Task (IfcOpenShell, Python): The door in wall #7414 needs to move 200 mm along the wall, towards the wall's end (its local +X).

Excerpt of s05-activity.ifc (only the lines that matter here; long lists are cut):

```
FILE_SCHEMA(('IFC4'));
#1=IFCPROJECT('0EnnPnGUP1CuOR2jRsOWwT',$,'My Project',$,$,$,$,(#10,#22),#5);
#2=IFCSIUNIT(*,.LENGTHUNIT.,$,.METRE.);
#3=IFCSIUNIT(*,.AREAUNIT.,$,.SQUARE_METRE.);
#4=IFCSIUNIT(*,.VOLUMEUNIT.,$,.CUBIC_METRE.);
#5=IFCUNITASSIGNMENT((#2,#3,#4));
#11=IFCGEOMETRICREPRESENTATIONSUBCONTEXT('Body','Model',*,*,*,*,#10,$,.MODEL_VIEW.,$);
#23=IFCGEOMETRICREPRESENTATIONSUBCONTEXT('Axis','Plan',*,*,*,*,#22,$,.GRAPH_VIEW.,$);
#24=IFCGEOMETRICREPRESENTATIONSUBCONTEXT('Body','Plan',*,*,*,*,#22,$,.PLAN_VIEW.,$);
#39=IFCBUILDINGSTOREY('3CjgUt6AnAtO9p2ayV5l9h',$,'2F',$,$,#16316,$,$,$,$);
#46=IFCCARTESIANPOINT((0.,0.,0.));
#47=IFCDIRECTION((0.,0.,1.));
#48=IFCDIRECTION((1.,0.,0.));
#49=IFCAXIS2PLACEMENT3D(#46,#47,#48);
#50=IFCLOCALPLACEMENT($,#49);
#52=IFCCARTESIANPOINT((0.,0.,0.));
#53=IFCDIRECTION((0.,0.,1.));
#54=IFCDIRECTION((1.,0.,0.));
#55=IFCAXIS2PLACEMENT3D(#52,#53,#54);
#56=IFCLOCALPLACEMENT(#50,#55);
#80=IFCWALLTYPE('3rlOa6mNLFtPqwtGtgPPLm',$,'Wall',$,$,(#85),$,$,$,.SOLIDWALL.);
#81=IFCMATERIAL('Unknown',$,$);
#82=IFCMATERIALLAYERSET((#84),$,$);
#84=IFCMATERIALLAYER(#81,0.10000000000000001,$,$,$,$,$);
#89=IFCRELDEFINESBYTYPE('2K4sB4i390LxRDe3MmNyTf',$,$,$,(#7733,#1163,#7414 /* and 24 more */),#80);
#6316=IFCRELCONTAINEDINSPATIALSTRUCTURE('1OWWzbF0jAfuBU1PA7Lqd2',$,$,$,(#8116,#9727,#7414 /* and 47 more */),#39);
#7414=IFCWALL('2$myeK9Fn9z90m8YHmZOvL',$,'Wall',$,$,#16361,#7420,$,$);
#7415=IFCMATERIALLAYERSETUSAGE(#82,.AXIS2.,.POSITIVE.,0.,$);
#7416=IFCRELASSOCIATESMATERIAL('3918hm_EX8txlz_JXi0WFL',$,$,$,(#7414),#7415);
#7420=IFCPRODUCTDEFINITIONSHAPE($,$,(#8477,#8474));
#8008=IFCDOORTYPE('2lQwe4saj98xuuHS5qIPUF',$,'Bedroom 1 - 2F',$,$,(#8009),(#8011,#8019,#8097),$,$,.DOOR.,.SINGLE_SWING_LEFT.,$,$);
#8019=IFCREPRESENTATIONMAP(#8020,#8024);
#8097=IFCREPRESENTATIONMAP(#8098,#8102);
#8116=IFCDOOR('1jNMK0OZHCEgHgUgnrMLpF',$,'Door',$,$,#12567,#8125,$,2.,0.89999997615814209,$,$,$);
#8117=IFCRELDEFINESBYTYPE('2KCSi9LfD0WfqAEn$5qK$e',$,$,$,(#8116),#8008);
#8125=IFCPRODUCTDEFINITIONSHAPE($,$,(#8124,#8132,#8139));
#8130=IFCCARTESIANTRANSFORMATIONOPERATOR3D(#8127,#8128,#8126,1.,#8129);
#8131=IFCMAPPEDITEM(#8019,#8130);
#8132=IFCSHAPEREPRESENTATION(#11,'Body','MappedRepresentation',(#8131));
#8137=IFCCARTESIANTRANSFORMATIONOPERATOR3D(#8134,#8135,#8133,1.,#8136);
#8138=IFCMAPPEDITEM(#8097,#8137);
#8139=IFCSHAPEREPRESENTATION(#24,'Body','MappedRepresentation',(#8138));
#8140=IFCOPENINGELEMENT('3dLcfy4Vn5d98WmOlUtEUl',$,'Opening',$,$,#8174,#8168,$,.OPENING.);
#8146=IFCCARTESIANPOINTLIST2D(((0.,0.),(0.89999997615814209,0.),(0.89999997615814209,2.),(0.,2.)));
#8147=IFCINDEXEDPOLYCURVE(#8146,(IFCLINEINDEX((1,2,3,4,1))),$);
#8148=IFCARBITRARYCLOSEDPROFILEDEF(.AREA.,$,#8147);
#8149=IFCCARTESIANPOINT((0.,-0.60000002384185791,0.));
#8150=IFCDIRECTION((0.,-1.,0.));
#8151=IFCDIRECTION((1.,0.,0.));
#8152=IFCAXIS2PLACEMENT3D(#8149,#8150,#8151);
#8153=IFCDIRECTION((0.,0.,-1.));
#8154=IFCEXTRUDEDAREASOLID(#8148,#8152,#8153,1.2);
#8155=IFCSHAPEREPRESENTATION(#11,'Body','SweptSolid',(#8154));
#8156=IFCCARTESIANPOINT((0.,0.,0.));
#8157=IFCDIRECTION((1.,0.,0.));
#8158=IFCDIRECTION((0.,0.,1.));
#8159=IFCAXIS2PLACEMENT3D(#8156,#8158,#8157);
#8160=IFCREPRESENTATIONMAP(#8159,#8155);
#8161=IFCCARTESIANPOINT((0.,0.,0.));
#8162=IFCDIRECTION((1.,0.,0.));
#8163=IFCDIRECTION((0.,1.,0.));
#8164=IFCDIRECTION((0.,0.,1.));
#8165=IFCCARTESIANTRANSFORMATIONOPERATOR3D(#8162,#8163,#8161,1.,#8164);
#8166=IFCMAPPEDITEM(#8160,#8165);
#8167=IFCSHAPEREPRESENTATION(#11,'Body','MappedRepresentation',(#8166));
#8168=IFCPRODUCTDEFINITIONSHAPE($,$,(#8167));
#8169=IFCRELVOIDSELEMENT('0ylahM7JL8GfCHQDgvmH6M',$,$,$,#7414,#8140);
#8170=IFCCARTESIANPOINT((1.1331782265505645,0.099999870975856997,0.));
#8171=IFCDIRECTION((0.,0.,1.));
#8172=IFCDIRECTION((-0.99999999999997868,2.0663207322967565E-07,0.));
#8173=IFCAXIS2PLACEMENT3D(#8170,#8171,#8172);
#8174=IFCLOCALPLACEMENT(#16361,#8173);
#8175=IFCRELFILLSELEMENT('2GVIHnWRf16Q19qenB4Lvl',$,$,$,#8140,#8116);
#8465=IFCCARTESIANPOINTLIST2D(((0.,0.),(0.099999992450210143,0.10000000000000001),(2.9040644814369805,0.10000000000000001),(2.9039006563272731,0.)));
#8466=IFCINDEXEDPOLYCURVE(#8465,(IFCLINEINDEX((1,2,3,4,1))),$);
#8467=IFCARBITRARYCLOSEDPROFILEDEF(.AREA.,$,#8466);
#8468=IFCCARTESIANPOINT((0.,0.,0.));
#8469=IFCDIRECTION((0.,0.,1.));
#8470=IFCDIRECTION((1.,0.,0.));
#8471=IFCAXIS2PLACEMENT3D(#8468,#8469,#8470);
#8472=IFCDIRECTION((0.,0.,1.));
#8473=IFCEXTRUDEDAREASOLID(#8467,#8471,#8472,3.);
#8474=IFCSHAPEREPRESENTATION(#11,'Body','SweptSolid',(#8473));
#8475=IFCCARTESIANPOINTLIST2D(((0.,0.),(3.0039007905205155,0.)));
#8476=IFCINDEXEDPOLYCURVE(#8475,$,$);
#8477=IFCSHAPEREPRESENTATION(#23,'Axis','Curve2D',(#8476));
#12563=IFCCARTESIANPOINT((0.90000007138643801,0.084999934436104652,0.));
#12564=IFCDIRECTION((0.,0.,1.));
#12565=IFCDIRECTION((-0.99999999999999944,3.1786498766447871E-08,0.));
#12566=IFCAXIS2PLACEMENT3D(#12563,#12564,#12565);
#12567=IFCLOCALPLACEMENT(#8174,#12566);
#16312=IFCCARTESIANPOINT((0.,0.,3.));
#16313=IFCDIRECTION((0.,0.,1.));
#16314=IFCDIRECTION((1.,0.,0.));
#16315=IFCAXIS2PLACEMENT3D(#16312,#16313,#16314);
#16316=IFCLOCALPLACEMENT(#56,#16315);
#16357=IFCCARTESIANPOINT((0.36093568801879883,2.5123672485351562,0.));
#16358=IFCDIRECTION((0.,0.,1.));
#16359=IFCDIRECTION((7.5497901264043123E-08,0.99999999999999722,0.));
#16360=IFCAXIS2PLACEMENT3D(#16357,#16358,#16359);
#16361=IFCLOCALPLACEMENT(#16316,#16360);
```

```python
import ifcopenshell
import ifcopenshell.api.geometry
import ifcopenshell.util.placement
import ifcopenshell.util.unit

model = ifcopenshell.open("s05-activity.ifc")
unit_scale = ifcopenshell.util.unit.calculate_unit_scale(model)

door = model.by_guid("1jNMK0OZHCEgHgUgnrMLpF")
opening = door.FillsVoids[0].RelatingOpeningElement
wall = opening.VoidsElements[0].RelatingBuildingElement

wall_matrix = ifcopenshell.util.placement.get_local_placement(wall.ObjectPlacement)
shift = wall_matrix[:3, 0] * 0.2 / unit_scale
before = ifcopenshell.util.placement.get_local_placement(door.ObjectPlacement)[:3, 3].copy()

# The door is placed relative to its opening, so it follows when the opening moves.
matrix = ifcopenshell.util.placement.get_local_placement(opening.ObjectPlacement)
matrix[:3, 3] += shift
ifcopenshell.api.geometry.edit_object_placement(
    model, product=opening, matrix=matrix, is_si=False, should_transform_children=True
)

after = ifcopenshell.util.placement.get_local_placement(door.ObjectPlacement)[:3, 3]
print("door moved by", (after - before).round(3) + 0.0)

model.write("s05-activity_edited.ifc")
```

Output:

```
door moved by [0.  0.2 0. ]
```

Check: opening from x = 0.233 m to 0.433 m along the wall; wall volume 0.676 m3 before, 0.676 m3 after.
